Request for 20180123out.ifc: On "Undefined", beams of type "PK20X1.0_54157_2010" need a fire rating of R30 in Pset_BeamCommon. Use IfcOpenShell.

First a look at what the model holds.

```python
import ifcopenshell
import ifcopenshell.util.element

model = ifcopenshell.open("20180123out.ifc")
print(model.schema)
storey = next(s for s in model.by_type("IfcBuildingStorey") if s.Name == "Undefined")
beams = [e for e in ifcopenshell.util.element.get_decomposition(storey) if e.is_a("IfcBeam")]
seen = {}
for e in beams:
    element_type = ifcopenshell.util.element.get_type(e)
    key = (element_type.Name if element_type != e and element_type else None, ifcopenshell.util.element.get_pset(e, "Pset_BeamCommon", "FireRating"))
    seen[key] = seen.get(key, 0) + 1
for (name, value), count in sorted(seen.items(), key=str):
    print(count, "x", name, "|", value)
```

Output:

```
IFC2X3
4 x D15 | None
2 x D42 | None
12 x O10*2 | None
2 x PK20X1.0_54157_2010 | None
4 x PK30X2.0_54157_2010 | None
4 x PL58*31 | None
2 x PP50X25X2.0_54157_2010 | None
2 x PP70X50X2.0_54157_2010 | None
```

```python
import ifcopenshell
import ifcopenshell.api.pset
import ifcopenshell.util.element

model = ifcopenshell.open("20180123out.ifc")

storey = next(s for s in model.by_type("IfcBuildingStorey") if s.Name == "Undefined")
beams = [e for e in ifcopenshell.util.element.get_decomposition(storey) if e.is_a("IfcBeam")]

count = 0
for e in beams:
    element_type = ifcopenshell.util.element.get_type(e)
    if element_type in (None, e) or element_type.Name != "PK20X1.0_54157_2010":
        continue
    found = ifcopenshell.util.element.get_pset(e, "Pset_BeamCommon", should_inherit=False)
    if found:
        pset = model.by_id(found["id"])
        if len(ifcopenshell.util.element.get_elements_by_pset(pset)) > 1:
            pset = ifcopenshell.api.pset.unshare_pset(model, products=[e], pset=pset)[0]
    else:
        pset = ifcopenshell.api.pset.add_pset(model, product=e, name="Pset_BeamCommon")
    ifcopenshell.api.pset.edit_pset(model, pset=pset, properties={"FireRating": "R30"})
    count += 1

print(count, "beams updated")

model.write("20180123out_rev.ifc")
```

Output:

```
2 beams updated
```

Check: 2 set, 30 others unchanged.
